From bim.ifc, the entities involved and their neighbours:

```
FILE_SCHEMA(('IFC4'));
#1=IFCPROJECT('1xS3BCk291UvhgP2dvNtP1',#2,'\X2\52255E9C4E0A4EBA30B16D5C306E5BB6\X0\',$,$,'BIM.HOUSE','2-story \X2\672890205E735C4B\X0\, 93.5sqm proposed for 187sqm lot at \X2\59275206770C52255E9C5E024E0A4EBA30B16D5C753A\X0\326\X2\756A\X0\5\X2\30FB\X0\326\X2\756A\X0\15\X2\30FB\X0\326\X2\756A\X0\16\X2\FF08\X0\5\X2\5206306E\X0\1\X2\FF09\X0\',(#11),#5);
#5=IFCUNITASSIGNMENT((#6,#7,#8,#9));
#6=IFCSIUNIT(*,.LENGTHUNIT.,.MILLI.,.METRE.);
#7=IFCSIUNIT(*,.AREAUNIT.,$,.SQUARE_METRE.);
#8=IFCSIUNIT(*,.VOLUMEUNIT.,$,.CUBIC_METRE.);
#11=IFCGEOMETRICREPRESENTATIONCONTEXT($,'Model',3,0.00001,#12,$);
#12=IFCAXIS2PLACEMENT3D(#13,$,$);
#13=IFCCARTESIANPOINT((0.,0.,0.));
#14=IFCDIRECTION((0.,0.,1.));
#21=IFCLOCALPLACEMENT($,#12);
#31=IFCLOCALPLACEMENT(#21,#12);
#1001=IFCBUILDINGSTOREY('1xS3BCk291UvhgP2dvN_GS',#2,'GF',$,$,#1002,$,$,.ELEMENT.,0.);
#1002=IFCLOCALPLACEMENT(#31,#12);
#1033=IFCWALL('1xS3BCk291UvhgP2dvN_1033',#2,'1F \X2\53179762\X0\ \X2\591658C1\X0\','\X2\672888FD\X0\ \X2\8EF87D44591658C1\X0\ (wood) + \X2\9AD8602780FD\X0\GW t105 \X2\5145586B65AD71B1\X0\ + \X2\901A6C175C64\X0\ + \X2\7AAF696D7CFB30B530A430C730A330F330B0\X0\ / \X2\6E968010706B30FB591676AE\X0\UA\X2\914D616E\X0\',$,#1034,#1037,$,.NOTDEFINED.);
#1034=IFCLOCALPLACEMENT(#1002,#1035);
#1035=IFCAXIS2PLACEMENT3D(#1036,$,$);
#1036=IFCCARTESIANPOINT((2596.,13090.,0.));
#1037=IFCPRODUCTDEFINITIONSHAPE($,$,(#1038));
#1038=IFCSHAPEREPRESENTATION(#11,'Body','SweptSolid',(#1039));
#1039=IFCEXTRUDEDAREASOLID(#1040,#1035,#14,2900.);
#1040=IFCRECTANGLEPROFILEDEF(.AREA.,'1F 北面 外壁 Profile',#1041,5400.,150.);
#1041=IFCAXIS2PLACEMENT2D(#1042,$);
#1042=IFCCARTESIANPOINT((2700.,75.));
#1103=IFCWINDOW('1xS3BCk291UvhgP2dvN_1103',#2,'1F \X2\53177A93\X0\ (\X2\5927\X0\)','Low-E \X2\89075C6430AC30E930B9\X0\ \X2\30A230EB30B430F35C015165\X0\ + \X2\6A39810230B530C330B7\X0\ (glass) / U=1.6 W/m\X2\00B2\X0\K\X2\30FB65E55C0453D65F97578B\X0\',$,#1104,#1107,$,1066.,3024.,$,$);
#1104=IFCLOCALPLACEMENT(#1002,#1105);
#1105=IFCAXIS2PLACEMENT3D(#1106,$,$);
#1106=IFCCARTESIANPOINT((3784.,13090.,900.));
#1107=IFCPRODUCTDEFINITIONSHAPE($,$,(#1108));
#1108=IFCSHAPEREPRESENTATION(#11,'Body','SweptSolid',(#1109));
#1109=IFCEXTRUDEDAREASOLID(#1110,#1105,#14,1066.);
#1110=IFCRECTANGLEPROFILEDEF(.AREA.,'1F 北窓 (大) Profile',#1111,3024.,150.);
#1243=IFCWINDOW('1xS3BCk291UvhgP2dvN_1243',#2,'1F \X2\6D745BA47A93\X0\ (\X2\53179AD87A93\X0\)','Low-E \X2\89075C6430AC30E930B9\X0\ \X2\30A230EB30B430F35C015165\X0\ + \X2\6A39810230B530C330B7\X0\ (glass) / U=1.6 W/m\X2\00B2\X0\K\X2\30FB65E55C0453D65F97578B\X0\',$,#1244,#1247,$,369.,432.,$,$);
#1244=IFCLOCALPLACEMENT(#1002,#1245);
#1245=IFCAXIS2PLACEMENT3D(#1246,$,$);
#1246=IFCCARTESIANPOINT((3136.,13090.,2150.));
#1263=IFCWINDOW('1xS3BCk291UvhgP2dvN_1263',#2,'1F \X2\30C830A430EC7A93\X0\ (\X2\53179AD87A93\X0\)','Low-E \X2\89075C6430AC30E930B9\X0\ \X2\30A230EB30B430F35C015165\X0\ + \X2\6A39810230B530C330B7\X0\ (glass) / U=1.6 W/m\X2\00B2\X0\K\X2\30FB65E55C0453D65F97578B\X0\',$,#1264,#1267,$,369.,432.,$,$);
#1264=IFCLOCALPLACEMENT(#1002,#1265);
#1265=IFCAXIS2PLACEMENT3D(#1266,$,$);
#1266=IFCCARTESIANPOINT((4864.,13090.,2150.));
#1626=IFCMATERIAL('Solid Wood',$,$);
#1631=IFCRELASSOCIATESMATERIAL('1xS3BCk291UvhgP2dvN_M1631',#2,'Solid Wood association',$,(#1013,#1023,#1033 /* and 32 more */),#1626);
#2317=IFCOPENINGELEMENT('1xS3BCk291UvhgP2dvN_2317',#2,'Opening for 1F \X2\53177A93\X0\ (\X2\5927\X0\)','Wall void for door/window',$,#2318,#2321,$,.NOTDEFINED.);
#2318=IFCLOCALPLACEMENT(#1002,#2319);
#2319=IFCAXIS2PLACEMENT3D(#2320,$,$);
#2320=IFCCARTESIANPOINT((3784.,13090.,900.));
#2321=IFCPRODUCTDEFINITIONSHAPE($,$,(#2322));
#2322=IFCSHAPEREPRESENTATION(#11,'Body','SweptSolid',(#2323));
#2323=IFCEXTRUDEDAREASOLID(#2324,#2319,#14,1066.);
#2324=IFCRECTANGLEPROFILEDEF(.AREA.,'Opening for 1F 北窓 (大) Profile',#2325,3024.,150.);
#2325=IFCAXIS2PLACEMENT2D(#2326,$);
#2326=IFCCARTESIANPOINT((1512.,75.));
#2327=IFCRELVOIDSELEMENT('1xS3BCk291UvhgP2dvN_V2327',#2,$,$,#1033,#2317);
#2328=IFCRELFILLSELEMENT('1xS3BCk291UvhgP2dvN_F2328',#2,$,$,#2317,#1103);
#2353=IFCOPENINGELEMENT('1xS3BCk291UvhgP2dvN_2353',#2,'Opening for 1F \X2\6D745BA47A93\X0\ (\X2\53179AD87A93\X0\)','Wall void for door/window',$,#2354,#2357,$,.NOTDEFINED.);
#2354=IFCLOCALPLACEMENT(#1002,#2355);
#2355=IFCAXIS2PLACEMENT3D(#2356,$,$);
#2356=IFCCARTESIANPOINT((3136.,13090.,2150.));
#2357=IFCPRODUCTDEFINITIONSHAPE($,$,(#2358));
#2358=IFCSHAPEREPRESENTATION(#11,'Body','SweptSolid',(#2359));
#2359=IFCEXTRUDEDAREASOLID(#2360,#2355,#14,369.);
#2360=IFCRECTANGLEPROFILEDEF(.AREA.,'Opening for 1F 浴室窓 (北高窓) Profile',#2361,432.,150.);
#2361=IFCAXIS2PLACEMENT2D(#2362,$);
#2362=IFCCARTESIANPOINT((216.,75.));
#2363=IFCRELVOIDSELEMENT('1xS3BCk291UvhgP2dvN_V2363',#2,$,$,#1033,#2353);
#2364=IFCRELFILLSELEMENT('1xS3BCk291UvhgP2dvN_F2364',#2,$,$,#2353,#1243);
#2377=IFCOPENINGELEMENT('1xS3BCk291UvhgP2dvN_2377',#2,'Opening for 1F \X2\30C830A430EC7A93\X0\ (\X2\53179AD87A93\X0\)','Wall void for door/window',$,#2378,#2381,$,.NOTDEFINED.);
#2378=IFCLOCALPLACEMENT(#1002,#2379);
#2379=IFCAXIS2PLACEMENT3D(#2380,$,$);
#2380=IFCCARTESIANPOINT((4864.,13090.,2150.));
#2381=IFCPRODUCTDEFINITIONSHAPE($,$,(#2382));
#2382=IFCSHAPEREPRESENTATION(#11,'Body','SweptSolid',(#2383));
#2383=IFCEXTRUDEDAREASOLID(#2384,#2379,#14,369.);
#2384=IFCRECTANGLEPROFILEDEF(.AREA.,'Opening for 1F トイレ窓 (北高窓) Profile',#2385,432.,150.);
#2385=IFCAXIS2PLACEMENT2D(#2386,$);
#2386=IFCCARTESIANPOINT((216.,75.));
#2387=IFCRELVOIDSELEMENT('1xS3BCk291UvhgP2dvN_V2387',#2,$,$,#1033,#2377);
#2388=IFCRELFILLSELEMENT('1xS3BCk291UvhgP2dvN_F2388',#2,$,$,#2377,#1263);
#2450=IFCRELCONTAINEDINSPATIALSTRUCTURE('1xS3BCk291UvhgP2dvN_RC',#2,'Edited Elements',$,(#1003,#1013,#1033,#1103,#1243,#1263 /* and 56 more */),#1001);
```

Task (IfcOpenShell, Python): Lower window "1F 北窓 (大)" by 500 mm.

```python
import numpy as np
import ifcopenshell
import ifcopenshell.api.geometry
import ifcopenshell.util.placement
import ifcopenshell.util.unit

model = ifcopenshell.open("bim.ifc")
unit_scale = ifcopenshell.util.unit.calculate_unit_scale(model)

window = model.by_guid("1xS3BCk291UvhgP2dvN_1103")
opening = window.FillsVoids[0].RelatingOpeningElement
dz = -500.0

shift = np.array([0.0, 0.0, dz])
# The window is not placed relative to its opening, so move both.
for product in (opening, window):
    matrix = ifcopenshell.util.placement.get_local_placement(product.ObjectPlacement)
    matrix[:3, 3] += shift
    ifcopenshell.api.geometry.edit_object_placement(model, product=product, matrix=matrix, is_si=False)

print(f"moved by {dz * unit_scale:+.3f} m")

model.write("bim_updated.ifc")
```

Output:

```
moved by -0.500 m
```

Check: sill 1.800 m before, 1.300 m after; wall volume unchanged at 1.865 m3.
